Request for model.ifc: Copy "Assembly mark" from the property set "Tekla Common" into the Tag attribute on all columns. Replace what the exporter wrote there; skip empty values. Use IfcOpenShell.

First a look at what the model holds.

```python
import ifcopenshell
import ifcopenshell.util.element

model = ifcopenshell.open("model.ifc")
print(model.schema)
columns = model.by_type("IfcColumn")
print(len(columns), "columns")
for e in columns[:8]:
    source = ifcopenshell.util.element.get_pset(e, "Tekla Common", "Assembly mark")
    target = e.Tag
    print(e.id(), repr(source), repr(target), sep=" | ")
```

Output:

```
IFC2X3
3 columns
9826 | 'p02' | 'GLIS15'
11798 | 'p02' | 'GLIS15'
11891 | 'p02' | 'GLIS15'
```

```python
import ifcopenshell
import ifcopenshell.util.element

model = ifcopenshell.open("model.ifc")

count = 0
for e in model.by_type("IfcColumn"):
    value = ifcopenshell.util.element.get_pset(e, "Tekla Common", "Assembly mark")
    current = e.Tag
    if not value or not value.strip() or current == value:
        continue
    e.Tag = value
    count += 1

print(count, "columns updated")

model.write("model_edited.ifc")
```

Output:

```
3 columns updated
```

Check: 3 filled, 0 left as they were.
